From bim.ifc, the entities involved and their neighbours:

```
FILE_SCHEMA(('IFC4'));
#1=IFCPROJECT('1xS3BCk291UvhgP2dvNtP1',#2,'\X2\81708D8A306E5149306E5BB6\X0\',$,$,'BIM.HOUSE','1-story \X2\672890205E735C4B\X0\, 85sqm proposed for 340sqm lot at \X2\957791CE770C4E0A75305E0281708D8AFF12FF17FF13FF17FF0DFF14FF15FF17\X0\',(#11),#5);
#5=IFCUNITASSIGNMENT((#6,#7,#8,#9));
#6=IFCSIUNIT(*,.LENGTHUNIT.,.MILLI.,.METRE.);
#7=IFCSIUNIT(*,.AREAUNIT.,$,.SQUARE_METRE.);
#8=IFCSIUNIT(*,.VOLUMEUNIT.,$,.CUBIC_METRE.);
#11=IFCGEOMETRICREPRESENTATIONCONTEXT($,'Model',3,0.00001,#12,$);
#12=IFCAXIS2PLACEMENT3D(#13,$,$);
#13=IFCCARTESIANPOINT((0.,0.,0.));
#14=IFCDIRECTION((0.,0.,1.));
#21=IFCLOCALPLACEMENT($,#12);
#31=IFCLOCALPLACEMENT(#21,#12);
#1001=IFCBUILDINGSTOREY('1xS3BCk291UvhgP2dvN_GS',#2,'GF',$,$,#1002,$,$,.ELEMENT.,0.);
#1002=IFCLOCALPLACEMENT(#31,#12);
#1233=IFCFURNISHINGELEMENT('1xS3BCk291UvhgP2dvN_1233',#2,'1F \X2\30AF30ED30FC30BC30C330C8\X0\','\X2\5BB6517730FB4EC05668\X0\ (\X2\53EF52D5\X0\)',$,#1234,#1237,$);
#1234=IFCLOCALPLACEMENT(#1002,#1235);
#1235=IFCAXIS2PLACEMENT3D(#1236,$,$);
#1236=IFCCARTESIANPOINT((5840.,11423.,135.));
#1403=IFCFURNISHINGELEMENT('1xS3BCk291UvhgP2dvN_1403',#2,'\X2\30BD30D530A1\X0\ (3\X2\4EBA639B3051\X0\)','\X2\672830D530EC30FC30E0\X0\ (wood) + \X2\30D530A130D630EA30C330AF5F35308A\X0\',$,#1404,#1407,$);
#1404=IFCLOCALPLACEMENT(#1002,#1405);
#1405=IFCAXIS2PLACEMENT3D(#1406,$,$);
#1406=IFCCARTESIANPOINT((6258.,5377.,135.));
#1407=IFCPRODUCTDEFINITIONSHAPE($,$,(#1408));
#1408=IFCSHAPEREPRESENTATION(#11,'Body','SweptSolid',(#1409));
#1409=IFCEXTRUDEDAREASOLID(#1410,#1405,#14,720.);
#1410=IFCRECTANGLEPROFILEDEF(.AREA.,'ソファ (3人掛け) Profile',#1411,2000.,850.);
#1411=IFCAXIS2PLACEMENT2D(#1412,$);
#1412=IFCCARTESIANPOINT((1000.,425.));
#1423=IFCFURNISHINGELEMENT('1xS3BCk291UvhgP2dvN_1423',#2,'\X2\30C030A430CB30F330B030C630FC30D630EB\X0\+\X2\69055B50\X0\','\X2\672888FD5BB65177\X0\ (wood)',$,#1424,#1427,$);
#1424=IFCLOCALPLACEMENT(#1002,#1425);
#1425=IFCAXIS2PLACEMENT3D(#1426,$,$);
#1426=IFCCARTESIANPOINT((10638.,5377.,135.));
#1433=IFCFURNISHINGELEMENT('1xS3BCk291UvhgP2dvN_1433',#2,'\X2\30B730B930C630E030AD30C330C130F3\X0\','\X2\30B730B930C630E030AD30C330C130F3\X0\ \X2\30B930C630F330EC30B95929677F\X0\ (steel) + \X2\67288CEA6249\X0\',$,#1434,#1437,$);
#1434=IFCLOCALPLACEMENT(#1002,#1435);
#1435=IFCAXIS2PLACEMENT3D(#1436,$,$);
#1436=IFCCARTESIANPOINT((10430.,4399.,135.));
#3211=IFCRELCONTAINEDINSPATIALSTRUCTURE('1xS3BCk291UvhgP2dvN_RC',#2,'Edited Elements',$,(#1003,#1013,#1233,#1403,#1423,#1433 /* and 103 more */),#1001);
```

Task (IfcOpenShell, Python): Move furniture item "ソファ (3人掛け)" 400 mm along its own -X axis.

```python
import ifcopenshell
import ifcopenshell.api.geometry
import ifcopenshell.util.placement
import ifcopenshell.util.unit

model = ifcopenshell.open("bim.ifc")
unit_scale = ifcopenshell.util.unit.calculate_unit_scale(model)

item = model.by_id(1403)
matrix = ifcopenshell.util.placement.get_local_placement(item.ObjectPlacement)
matrix[:3, 3] -= matrix[:3, 0] * 0.4 / unit_scale
ifcopenshell.api.geometry.edit_object_placement(model, product=item, matrix=matrix, is_si=False)

print(ifcopenshell.util.placement.get_local_placement(item.ObjectPlacement).round(3) + 0.0)

model.write("bim_rev.ifc")
```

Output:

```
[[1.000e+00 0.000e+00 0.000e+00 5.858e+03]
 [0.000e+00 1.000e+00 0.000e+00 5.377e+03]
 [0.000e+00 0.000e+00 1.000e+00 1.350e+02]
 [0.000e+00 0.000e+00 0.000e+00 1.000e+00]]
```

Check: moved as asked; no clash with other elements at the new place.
